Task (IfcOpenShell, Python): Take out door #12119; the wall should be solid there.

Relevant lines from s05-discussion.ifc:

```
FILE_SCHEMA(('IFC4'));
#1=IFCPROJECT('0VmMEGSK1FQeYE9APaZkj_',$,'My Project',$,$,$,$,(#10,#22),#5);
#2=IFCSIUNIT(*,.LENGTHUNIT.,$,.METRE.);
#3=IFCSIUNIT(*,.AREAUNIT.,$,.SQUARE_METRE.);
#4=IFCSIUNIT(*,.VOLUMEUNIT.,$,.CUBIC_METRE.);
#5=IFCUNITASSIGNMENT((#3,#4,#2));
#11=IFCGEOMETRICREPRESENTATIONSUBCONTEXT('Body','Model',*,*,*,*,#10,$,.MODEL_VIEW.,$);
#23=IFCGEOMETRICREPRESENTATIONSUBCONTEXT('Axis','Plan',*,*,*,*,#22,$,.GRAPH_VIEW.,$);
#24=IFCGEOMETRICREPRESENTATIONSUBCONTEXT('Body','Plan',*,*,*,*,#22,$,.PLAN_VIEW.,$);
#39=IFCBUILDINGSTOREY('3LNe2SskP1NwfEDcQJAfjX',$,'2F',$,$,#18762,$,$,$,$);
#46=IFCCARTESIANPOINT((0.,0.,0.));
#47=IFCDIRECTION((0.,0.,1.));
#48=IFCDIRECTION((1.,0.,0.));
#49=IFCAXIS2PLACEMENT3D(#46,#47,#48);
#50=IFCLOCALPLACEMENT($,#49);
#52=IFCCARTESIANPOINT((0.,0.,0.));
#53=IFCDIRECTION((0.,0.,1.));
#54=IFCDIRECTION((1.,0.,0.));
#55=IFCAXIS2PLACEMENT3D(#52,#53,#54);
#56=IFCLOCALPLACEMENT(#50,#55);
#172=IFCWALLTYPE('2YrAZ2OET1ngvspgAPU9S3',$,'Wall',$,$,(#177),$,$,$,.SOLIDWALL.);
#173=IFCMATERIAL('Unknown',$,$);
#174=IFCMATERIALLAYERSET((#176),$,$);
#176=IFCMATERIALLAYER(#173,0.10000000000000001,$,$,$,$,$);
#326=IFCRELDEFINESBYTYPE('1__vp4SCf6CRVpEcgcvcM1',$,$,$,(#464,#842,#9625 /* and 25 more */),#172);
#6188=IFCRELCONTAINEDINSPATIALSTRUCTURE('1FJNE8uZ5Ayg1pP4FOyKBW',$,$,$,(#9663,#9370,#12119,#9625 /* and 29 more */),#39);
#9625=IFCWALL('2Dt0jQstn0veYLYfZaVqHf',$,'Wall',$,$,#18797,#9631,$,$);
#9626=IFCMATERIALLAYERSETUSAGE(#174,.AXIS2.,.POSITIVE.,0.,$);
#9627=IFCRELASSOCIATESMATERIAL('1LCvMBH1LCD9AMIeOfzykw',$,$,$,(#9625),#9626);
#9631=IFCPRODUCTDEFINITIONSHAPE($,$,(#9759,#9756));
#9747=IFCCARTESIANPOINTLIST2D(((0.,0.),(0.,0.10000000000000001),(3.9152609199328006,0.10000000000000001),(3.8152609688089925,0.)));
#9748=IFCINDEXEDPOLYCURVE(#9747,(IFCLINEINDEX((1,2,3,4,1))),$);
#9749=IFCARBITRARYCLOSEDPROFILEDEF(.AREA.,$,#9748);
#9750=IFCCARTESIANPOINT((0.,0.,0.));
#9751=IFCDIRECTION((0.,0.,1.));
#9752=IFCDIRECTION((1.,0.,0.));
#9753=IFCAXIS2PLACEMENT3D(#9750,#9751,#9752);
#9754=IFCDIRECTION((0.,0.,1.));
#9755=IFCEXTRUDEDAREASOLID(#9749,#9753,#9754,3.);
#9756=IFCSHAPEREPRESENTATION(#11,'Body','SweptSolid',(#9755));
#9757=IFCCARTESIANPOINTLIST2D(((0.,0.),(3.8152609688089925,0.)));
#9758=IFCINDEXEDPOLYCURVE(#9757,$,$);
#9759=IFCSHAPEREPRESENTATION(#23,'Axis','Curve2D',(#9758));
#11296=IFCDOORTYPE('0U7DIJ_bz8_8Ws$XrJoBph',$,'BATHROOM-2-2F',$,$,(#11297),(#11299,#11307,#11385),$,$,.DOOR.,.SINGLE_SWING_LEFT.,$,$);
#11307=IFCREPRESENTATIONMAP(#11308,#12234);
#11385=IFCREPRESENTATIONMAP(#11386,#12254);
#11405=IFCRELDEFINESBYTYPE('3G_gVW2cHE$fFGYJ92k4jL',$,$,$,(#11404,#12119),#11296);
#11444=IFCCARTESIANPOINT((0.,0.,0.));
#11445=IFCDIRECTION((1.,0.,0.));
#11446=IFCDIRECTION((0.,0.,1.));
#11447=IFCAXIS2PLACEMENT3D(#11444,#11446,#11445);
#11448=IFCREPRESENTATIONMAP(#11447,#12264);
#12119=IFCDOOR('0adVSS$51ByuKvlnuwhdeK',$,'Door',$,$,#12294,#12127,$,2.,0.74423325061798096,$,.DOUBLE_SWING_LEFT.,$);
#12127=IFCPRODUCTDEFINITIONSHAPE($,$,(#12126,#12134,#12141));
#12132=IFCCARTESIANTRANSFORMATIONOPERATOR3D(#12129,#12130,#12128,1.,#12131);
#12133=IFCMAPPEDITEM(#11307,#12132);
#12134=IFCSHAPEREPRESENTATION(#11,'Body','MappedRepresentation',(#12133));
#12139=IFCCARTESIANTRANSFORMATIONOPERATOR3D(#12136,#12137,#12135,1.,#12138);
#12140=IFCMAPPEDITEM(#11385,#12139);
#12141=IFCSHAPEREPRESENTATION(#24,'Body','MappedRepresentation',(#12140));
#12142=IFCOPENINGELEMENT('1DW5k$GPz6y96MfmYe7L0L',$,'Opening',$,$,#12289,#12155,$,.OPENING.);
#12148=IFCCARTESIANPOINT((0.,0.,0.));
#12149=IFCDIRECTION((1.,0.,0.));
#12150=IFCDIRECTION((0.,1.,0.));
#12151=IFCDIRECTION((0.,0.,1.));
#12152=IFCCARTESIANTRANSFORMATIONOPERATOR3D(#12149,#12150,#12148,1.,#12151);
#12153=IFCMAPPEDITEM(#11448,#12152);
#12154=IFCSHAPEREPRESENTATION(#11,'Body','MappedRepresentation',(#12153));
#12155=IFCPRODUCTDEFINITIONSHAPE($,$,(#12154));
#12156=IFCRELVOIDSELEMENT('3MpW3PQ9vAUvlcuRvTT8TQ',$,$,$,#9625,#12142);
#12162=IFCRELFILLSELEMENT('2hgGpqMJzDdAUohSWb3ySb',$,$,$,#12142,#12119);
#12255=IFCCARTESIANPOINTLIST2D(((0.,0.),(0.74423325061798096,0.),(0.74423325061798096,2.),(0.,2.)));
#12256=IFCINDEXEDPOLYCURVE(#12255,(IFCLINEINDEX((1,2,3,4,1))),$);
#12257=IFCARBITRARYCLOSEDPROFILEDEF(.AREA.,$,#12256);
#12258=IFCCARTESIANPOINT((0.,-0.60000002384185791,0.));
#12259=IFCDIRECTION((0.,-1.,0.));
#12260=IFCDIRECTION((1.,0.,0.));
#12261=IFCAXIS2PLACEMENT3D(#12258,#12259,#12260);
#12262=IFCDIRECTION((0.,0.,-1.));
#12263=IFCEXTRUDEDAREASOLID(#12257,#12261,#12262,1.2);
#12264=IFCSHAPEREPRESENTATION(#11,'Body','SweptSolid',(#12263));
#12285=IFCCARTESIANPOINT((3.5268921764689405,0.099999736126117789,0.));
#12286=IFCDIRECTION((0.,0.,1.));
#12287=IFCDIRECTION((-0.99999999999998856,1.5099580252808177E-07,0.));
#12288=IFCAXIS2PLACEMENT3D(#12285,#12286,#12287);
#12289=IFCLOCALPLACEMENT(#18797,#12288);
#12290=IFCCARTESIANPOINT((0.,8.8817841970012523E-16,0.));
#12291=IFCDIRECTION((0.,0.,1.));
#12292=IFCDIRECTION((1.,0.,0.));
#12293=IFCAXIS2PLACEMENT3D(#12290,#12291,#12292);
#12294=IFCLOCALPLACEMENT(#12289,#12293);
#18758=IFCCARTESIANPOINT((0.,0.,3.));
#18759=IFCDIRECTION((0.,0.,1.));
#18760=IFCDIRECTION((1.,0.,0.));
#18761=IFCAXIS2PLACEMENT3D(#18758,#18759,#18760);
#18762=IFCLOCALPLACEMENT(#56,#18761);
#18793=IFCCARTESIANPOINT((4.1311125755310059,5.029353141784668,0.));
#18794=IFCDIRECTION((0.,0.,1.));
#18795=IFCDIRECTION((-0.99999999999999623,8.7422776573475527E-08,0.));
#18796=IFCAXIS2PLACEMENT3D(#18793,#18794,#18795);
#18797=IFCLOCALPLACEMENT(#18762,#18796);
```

```python
import ifcopenshell
import ifcopenshell.api.feature
import ifcopenshell.api.root
import ifcopenshell.geom
import ifcopenshell.util.shape

model = ifcopenshell.open("s05-discussion.ifc")
settings = ifcopenshell.geom.settings()


def volume(element):
    """Net volume in cubic metres, openings subtracted."""
    shape = ifcopenshell.geom.create_shape(settings, element)
    return ifcopenshell.util.shape.get_volume(shape.geometry)


door = model.by_id(12119)
opening = door.FillsVoids[0].RelatingOpeningElement
wall = opening.VoidsElements[0].RelatingBuildingElement
before = volume(wall)

ifcopenshell.api.root.remove_product(model, product=door)
ifcopenshell.api.feature.remove_feature(model, feature=opening)

after = volume(wall)

print(f"wall volume {before:.3f} -> {after:.3f} m3")

model.write("s05-discussion_rev.ifc")
```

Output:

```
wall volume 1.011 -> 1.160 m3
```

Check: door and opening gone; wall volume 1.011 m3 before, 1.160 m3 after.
